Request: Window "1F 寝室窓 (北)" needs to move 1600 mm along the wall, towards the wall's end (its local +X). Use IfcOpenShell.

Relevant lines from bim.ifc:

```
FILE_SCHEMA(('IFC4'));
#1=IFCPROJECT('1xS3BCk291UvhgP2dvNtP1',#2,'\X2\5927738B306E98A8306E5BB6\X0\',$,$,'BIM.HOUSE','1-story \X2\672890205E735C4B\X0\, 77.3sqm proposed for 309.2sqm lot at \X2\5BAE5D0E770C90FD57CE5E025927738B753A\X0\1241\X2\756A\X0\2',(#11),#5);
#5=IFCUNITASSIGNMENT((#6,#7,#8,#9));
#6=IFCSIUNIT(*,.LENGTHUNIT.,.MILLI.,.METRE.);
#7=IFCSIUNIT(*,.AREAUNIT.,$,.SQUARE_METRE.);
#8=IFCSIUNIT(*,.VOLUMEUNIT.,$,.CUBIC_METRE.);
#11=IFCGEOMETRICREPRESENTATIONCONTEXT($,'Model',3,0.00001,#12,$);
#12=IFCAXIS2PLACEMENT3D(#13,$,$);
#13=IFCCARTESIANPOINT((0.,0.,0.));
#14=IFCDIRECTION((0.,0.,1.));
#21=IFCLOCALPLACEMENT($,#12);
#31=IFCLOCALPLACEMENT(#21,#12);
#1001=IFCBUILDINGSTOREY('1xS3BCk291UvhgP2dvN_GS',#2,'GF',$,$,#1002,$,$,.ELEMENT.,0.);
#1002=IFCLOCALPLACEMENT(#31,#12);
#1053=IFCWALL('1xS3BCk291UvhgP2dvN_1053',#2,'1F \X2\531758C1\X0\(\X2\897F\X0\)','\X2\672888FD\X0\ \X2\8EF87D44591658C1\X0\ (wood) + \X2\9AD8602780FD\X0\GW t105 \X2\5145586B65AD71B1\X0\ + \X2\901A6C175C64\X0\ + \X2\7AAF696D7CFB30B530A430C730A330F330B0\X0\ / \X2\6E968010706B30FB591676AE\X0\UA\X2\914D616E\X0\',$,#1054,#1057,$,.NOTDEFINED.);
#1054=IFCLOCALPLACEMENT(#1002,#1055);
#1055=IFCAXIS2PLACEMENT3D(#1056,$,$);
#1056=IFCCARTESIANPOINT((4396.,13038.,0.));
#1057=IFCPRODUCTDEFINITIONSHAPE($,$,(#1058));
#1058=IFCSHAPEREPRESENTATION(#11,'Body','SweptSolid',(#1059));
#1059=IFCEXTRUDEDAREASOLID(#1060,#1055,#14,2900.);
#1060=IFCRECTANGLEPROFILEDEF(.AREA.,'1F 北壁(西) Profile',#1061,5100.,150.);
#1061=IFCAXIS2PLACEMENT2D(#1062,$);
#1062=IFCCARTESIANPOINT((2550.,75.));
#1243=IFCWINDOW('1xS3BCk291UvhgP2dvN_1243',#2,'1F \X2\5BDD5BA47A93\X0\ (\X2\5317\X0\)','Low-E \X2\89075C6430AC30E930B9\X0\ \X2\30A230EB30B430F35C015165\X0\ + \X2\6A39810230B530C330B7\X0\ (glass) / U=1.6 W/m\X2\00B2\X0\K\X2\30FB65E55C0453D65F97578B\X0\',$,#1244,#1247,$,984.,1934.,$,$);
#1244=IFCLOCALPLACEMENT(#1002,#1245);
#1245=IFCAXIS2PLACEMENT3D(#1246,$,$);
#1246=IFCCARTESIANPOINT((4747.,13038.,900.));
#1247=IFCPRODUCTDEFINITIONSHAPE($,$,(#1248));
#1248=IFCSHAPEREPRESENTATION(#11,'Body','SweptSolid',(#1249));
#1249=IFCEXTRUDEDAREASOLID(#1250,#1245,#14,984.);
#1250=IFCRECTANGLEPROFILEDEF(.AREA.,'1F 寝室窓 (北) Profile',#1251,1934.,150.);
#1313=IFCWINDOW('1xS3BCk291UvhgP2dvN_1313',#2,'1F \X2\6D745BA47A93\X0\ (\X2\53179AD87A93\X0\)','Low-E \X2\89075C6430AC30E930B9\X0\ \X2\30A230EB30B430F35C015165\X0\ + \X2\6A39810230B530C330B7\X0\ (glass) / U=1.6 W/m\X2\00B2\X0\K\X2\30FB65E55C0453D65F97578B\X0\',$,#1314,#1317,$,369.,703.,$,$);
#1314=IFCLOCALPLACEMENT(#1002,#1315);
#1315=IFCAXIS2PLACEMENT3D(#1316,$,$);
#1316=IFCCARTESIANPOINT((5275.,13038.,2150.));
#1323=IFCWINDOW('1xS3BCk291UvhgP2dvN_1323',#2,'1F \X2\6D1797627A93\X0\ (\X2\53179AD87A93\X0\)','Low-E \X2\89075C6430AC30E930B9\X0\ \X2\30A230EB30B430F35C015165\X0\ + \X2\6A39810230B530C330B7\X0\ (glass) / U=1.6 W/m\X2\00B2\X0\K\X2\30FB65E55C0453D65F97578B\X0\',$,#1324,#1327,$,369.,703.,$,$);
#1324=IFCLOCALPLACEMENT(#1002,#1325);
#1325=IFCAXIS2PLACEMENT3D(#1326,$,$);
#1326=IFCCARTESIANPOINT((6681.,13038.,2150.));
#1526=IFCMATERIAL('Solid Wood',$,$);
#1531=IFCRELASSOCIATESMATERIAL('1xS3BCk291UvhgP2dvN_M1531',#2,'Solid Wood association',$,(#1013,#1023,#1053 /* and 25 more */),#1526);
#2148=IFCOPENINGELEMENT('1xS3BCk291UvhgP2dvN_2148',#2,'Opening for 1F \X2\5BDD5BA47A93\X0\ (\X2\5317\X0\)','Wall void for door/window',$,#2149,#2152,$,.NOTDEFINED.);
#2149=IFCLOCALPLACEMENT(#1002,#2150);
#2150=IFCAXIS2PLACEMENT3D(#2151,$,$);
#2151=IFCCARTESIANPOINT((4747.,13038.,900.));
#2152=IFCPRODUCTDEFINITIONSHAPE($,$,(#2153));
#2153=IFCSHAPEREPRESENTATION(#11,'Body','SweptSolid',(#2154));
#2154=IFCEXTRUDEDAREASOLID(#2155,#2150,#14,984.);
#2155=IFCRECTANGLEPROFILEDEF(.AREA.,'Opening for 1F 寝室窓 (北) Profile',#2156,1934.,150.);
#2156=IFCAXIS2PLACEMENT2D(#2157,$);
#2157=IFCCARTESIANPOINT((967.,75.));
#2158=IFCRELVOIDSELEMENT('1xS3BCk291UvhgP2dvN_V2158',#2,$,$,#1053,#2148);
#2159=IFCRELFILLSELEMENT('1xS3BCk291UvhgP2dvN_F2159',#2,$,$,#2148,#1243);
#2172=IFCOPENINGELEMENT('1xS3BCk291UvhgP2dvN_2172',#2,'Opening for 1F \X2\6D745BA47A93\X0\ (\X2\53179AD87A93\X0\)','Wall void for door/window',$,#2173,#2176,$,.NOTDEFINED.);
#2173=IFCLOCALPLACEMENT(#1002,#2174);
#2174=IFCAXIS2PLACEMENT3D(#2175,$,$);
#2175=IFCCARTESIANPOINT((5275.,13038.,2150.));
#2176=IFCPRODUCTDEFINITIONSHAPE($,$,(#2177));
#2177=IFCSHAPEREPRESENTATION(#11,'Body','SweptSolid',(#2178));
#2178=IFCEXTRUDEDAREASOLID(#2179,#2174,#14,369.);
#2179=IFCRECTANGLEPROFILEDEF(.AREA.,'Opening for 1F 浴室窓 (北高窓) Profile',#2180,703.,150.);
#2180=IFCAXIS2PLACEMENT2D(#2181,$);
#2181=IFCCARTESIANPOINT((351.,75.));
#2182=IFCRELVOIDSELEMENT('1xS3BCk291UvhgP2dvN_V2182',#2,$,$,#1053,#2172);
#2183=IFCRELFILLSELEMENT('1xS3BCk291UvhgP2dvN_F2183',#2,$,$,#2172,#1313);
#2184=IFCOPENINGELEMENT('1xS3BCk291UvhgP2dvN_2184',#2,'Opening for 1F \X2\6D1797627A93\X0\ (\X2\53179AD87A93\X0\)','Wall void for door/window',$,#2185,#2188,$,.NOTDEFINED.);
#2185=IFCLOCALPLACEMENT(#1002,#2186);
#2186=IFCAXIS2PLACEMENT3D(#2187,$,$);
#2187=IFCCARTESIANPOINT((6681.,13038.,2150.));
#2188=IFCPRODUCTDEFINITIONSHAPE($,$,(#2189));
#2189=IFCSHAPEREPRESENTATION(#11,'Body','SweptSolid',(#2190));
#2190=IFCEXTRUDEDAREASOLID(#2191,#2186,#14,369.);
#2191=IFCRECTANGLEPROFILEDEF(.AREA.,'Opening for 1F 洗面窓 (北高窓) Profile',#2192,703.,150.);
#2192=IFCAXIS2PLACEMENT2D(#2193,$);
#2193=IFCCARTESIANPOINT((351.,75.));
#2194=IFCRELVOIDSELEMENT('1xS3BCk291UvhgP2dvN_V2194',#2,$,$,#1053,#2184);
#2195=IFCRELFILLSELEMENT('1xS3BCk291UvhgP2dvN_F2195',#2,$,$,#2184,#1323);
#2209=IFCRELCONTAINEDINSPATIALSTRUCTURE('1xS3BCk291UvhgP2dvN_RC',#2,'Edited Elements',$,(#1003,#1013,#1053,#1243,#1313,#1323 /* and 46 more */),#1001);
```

```python
import ifcopenshell
import ifcopenshell.api.geometry
import ifcopenshell.util.placement

model = ifcopenshell.open("bim.ifc")

window = model.by_guid("1xS3BCk291UvhgP2dvN_1243")
opening = window.FillsVoids[0].RelatingOpeningElement
wall = opening.VoidsElements[0].RelatingBuildingElement

wall_matrix = ifcopenshell.util.placement.get_local_placement(wall.ObjectPlacement)
shift = wall_matrix[:3, 0] * 1600.0
before = ifcopenshell.util.placement.get_local_placement(window.ObjectPlacement)[:3, 3].copy()

# The window is not placed relative to its opening, so move both.
for product in (opening, window):
    matrix = ifcopenshell.util.placement.get_local_placement(product.ObjectPlacement)
    matrix[:3, 3] += shift
    ifcopenshell.api.geometry.edit_object_placement(model, product=product, matrix=matrix, is_si=False)

after = ifcopenshell.util.placement.get_local_placement(window.ObjectPlacement)[:3, 3]
print("window moved by", (after - before).round(3) + 0.0)

model.write("bim_rev.ifc")
```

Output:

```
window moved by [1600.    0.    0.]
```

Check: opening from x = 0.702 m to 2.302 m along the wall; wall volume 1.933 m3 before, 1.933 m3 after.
